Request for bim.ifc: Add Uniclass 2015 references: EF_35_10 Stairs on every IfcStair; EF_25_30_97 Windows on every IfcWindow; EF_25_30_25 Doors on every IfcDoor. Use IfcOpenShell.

First a look at what the model holds.

```python
import ifcopenshell

model = ifcopenshell.open("bim.ifc")
print(model.schema)
print("classifications:", [c.Name for c in model.by_type("IfcClassification")])
for ifc_class in ("IfcDoor", "IfcRoof", "IfcStair", "IfcWall", "IfcWindow"):
    print(ifc_class, len(model.by_type(ifc_class)))
```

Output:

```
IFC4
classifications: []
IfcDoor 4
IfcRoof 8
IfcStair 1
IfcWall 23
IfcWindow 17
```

```python
import ifcopenshell
import ifcopenshell.api.classification

model = ifcopenshell.open("bim.ifc")

system = ifcopenshell.api.classification.add_classification(model, classification="Uniclass 2015")

codes = {
    "IfcStair": ("EF_35_10", "Stairs"),
    "IfcWindow": ("EF_25_30_97", "Windows"),
    "IfcDoor": ("EF_25_30_25", "Doors"),
}
for ifc_class, (code, name) in codes.items():
    products = model.by_type(ifc_class)
    ifcopenshell.api.classification.add_reference(
        model, products=products, classification=system, identification=code, name=name
    )
    print(code, len(products))

model.write("bim_v2.ifc")
```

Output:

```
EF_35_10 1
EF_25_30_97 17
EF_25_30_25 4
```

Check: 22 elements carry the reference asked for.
